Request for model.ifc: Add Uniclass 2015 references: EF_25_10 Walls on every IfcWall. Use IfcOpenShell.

First a look at what the model holds.

```python
import ifcopenshell

model = ifcopenshell.open("model.ifc")
print(model.schema)
print("classifications:", [c.Name for c in model.by_type("IfcClassification")])
for ifc_class in ("IfcDoor", "IfcRoof", "IfcStair", "IfcWall", "IfcWindow"):
    print(ifc_class, len(model.by_type(ifc_class)))
```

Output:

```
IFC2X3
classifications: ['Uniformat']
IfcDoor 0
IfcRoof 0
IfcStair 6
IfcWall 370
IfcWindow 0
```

```python
import ifcopenshell
import ifcopenshell.api.classification

model = ifcopenshell.open("model.ifc")

# IFC2X3 requires Source and Edition and has no link from the project to the system.
system = model.create_entity("IfcClassification", Source="NBS", Edition="2015", Name="Uniclass 2015")

codes = {
    "IfcWall": ("EF_25_10", "Walls"),
}
for ifc_class, (code, name) in codes.items():
    products = model.by_type(ifc_class)
    ifcopenshell.api.classification.add_reference(
        model, products=products, classification=system, identification=code, name=name
    )
    print(code, len(products))

model.write("model_updated.ifc")
```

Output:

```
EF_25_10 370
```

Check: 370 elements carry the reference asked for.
